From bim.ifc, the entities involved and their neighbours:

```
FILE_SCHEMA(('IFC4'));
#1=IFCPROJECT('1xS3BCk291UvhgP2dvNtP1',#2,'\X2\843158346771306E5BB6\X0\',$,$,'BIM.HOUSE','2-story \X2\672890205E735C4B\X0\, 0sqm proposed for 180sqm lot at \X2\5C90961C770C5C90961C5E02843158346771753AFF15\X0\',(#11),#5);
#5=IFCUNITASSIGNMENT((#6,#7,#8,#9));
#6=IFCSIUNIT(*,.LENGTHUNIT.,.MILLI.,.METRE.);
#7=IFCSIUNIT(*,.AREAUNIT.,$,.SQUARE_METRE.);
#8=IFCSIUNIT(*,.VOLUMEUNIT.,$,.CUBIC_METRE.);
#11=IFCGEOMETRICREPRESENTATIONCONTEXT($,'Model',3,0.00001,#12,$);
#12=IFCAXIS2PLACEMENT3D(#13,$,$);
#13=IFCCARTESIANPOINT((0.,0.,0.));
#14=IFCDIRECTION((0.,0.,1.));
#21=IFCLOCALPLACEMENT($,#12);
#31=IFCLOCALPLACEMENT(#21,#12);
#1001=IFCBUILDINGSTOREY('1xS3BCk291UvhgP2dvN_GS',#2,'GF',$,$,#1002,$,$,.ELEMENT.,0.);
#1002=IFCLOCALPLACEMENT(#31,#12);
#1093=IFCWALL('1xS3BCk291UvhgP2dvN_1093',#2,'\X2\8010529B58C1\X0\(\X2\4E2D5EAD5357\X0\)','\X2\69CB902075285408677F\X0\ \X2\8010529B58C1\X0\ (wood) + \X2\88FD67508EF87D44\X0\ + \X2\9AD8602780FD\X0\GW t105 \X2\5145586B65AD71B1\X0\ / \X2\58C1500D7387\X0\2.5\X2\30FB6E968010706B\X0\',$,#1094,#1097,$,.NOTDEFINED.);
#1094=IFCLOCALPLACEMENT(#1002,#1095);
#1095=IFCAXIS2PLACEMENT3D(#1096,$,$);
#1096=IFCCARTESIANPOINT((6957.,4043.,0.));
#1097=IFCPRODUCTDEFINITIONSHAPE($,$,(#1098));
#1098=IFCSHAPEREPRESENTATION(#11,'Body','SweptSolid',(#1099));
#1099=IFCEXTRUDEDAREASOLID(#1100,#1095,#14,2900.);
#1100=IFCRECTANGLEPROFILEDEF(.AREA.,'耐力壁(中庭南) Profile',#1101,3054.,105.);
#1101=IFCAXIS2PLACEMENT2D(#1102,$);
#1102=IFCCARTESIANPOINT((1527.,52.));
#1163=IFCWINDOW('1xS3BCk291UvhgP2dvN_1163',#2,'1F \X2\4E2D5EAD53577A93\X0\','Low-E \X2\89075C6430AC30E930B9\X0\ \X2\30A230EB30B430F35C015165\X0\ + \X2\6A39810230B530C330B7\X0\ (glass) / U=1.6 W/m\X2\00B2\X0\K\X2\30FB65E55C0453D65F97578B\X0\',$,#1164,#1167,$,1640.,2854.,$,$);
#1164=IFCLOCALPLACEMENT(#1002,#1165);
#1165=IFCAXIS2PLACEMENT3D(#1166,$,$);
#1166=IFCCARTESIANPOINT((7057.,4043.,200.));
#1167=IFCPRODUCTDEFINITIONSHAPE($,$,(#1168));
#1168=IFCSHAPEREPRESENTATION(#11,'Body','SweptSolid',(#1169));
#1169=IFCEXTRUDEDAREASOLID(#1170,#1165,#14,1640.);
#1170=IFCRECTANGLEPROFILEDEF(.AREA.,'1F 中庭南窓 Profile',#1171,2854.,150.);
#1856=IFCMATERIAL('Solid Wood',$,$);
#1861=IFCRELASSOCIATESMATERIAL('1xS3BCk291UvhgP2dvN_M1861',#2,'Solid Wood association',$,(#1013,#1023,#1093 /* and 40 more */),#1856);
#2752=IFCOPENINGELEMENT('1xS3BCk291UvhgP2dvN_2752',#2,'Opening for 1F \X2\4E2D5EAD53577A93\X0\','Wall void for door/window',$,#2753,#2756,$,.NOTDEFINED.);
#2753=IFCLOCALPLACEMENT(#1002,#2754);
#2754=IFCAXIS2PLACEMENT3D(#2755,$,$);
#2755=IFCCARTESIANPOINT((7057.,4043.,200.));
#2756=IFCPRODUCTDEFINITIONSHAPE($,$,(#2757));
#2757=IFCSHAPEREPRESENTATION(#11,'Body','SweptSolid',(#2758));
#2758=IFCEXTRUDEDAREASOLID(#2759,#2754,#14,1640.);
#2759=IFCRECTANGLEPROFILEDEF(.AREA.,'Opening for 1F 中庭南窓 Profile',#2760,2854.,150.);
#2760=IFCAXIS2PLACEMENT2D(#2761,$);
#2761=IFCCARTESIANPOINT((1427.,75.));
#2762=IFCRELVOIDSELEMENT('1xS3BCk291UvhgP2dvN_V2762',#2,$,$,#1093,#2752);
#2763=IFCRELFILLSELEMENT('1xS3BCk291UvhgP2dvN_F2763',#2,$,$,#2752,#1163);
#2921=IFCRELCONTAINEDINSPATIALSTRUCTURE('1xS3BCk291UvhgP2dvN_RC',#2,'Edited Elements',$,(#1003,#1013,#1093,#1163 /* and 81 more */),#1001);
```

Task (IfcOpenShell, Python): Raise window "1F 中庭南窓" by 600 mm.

```python
import numpy as np
import ifcopenshell
import ifcopenshell.api.geometry
import ifcopenshell.util.placement
import ifcopenshell.util.unit

model = ifcopenshell.open("bim.ifc")
unit_scale = ifcopenshell.util.unit.calculate_unit_scale(model)

window = model.by_id(1163)
opening = window.FillsVoids[0].RelatingOpeningElement
dz = 0.6 / unit_scale

shift = np.array([0.0, 0.0, dz])
# The window is not placed relative to its opening, so move both.
for product in (opening, window):
    matrix = ifcopenshell.util.placement.get_local_placement(product.ObjectPlacement)
    matrix[:3, 3] += shift
    ifcopenshell.api.geometry.edit_object_placement(model, product=product, matrix=matrix, is_si=False)

print(f"moved by {dz * unit_scale:+.3f} m")

model.write("bim_rev.ifc")
```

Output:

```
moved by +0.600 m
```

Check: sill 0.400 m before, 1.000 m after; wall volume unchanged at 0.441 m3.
